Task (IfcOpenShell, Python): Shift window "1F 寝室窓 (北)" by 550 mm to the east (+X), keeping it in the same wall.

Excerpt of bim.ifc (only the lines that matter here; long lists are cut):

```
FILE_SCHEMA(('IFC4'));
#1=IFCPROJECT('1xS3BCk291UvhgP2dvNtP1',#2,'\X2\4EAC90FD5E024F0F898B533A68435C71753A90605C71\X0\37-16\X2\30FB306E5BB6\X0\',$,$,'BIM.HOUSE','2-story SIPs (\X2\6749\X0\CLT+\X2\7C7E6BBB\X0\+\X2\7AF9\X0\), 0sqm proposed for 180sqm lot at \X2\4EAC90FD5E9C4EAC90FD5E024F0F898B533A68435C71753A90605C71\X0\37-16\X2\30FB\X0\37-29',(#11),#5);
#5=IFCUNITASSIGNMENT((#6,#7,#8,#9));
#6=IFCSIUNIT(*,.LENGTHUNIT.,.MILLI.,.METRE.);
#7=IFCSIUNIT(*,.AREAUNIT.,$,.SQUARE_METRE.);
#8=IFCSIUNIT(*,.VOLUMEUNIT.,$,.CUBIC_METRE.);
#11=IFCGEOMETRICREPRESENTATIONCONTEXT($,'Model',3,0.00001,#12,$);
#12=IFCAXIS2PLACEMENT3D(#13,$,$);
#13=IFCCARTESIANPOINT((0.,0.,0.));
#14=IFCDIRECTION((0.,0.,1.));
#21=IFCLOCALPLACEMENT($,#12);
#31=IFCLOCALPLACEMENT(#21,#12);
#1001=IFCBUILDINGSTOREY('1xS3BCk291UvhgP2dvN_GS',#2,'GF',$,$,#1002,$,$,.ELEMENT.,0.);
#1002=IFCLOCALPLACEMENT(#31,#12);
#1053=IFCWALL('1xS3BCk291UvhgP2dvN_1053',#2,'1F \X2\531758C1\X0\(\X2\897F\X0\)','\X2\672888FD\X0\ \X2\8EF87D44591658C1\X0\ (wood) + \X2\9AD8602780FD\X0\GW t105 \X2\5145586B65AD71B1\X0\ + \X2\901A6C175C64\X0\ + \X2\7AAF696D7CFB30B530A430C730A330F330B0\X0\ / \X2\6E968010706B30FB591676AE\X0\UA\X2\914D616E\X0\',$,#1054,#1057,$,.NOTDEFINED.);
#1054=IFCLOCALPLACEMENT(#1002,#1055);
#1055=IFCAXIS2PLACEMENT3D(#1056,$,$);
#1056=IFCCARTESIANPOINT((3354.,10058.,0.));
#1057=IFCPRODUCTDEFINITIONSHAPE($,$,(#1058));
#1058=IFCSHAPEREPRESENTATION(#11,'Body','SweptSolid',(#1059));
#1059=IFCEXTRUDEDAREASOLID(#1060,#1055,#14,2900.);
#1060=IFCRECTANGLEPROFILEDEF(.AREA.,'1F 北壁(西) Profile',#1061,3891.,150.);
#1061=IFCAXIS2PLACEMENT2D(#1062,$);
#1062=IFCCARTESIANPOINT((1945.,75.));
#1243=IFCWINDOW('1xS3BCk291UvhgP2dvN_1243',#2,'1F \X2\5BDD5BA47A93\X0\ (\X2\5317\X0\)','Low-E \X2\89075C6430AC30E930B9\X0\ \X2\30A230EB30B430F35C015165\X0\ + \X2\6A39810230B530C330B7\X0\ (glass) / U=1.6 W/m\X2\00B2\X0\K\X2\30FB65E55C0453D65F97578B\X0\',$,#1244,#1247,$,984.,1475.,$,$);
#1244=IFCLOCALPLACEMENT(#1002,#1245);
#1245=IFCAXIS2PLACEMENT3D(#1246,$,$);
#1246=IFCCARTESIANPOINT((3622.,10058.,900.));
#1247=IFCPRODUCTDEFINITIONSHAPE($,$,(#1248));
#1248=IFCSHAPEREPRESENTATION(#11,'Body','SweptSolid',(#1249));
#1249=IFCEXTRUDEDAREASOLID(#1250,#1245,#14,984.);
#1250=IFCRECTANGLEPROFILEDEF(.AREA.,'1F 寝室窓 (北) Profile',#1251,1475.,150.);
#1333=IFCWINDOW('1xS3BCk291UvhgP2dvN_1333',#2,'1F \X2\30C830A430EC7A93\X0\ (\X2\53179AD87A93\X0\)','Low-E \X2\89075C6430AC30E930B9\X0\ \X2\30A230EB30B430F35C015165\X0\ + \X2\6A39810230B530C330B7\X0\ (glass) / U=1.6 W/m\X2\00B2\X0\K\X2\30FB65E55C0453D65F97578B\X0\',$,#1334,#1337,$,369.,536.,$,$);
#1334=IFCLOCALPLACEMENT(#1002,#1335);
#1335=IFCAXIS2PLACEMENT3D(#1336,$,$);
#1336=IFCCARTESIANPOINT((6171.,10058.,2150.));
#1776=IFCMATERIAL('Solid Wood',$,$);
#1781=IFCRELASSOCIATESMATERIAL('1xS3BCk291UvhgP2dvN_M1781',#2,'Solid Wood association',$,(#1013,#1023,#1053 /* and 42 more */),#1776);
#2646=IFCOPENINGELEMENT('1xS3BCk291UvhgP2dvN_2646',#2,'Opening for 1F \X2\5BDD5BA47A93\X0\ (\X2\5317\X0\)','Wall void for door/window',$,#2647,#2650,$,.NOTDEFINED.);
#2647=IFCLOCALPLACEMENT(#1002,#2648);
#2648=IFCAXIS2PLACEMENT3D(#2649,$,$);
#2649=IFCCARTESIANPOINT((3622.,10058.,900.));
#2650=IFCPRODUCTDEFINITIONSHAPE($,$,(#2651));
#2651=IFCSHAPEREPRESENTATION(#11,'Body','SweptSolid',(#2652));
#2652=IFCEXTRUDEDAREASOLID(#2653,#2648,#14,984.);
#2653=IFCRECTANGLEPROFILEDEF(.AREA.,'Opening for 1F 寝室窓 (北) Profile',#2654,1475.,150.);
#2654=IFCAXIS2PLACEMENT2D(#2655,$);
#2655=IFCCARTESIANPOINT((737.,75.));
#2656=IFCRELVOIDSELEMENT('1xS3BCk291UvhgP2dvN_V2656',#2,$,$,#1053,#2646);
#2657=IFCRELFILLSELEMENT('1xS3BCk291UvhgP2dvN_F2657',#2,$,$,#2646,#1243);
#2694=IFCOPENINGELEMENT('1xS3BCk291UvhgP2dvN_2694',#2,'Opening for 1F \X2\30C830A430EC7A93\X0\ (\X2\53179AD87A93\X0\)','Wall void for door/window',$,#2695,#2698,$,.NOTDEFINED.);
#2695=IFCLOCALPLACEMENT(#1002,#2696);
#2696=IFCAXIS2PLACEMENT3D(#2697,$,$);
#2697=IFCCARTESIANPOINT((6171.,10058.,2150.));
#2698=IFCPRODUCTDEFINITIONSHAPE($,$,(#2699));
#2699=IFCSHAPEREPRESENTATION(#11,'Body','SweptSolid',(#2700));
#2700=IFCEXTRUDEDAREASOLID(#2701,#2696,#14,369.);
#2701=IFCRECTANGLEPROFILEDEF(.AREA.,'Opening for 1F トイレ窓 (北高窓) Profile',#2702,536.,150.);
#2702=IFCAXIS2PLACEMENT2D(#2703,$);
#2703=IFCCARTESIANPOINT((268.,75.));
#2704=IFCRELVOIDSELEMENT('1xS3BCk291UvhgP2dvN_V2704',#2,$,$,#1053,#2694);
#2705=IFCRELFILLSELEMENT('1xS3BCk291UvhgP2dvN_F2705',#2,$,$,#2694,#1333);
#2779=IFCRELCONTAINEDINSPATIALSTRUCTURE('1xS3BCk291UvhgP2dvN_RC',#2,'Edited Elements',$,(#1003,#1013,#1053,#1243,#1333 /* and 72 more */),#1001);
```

```python
import ifcopenshell
import ifcopenshell.api.geometry
import ifcopenshell.util.placement
import ifcopenshell.util.unit

model = ifcopenshell.open("bim.ifc")
unit_scale = ifcopenshell.util.unit.calculate_unit_scale(model)

window = model.by_guid("1xS3BCk291UvhgP2dvN_1243")
opening = window.FillsVoids[0].RelatingOpeningElement
wall = opening.VoidsElements[0].RelatingBuildingElement

wall_matrix = ifcopenshell.util.placement.get_local_placement(wall.ObjectPlacement)
shift = wall_matrix[:3, 0] * 0.55 / unit_scale
before = ifcopenshell.util.placement.get_local_placement(window.ObjectPlacement)[:3, 3].copy()

# The window is not placed relative to its opening, so move both.
for product in (opening, window):
    matrix = ifcopenshell.util.placement.get_local_placement(product.ObjectPlacement)
    matrix[:3, 3] += shift
    ifcopenshell.api.geometry.edit_object_placement(model, product=product, matrix=matrix, is_si=False)

after = ifcopenshell.util.placement.get_local_placement(window.ObjectPlacement)[:3, 3]
print("window moved by", (after - before).round(3) + 0.0)

model.write("bim_rev.ifc")
```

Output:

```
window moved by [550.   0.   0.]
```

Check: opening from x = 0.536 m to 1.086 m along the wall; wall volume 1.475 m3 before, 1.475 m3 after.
